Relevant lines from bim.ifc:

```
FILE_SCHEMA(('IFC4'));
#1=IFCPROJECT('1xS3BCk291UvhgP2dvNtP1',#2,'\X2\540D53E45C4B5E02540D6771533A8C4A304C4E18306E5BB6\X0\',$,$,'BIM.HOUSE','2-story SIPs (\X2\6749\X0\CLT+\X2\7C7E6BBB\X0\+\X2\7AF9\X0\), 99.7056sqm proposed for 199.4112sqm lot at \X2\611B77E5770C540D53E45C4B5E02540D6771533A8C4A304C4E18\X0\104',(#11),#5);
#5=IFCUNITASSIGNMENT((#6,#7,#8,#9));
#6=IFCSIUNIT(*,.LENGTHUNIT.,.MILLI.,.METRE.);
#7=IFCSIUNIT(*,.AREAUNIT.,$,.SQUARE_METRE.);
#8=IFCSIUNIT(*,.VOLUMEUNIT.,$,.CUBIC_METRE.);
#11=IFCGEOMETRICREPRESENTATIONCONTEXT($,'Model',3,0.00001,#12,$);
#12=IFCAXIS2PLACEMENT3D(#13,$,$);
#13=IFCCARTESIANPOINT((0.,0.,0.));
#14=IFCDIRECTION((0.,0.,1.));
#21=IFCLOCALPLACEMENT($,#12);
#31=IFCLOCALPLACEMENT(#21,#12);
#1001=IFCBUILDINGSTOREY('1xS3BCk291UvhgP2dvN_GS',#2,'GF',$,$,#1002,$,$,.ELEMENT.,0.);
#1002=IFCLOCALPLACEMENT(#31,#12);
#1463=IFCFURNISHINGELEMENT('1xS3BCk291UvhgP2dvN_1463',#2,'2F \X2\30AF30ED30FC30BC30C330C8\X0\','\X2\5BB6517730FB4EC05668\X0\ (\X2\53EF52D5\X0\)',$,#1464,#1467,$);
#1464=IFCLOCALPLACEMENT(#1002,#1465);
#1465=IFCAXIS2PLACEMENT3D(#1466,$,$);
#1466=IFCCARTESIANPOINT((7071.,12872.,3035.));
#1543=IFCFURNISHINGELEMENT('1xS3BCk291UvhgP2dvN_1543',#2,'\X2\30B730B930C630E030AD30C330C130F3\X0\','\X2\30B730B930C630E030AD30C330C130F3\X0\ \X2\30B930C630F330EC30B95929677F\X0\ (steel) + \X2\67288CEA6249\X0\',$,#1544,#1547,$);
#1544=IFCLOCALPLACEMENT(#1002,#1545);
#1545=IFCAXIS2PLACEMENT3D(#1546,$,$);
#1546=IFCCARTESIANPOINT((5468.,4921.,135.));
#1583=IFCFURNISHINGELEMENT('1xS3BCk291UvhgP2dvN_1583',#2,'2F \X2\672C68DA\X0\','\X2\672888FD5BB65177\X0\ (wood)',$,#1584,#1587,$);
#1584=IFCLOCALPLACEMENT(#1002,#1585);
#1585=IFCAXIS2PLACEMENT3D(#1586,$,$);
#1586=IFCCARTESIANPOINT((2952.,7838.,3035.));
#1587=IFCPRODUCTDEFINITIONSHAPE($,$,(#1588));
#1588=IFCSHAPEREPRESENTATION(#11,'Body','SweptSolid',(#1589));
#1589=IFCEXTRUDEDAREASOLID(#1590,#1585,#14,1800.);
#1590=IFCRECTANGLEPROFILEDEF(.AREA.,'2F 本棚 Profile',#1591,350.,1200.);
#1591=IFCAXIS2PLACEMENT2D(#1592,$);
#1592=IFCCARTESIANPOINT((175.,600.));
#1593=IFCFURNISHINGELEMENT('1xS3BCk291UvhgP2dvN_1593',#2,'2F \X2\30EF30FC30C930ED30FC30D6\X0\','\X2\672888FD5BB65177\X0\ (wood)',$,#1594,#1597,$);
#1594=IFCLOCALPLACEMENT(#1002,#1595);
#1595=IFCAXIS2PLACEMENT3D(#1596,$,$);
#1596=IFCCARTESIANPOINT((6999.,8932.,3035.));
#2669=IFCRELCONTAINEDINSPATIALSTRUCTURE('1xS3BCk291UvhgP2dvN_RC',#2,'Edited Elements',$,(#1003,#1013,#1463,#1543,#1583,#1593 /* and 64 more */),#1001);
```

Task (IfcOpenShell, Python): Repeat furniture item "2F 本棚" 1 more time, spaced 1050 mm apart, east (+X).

```python
import numpy as np
import ifcopenshell
import ifcopenshell.api.geometry
import ifcopenshell.api.root
import ifcopenshell.util.element
import ifcopenshell.util.placement

model = ifcopenshell.open("bim.ifc")


def reuse_history(source, copy):
    """copy_class also copies each property set's owner history, people and application; keep the originals."""
    for rel in copy.IsDefinedBy:
        if rel.is_a("IfcRelDefinesByProperties") and (history := rel.RelatingPropertyDefinition.OwnerHistory):
            rel.RelatingPropertyDefinition.OwnerHistory = source.OwnerHistory
            ifcopenshell.util.element.remove_deep2(model, history)


source = model.by_guid("1xS3BCk291UvhgP2dvN_1583")
base = ifcopenshell.util.placement.get_local_placement(source.ObjectPlacement)
step = np.array([1.0, 0.0, 0.0]) * 1050.0

for i in range(1, 2):
    copy = ifcopenshell.api.root.copy_class(model, product=source)
    copy.Representation = ifcopenshell.util.element.copy_deep(
        model, source.Representation, exclude=["IfcGeometricRepresentationContext", "IfcRepresentationMap"]
    )
    reuse_history(source, copy)
    matrix = base.copy()
    matrix[:3, 3] += i * step
    print("added at", matrix[:3, 3].round(3) + 0.0)
    ifcopenshell.api.geometry.edit_object_placement(model, product=copy, matrix=matrix, is_si=False)

model.write("bim_v2.ifc")
```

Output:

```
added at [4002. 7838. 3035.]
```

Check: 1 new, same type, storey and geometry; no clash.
